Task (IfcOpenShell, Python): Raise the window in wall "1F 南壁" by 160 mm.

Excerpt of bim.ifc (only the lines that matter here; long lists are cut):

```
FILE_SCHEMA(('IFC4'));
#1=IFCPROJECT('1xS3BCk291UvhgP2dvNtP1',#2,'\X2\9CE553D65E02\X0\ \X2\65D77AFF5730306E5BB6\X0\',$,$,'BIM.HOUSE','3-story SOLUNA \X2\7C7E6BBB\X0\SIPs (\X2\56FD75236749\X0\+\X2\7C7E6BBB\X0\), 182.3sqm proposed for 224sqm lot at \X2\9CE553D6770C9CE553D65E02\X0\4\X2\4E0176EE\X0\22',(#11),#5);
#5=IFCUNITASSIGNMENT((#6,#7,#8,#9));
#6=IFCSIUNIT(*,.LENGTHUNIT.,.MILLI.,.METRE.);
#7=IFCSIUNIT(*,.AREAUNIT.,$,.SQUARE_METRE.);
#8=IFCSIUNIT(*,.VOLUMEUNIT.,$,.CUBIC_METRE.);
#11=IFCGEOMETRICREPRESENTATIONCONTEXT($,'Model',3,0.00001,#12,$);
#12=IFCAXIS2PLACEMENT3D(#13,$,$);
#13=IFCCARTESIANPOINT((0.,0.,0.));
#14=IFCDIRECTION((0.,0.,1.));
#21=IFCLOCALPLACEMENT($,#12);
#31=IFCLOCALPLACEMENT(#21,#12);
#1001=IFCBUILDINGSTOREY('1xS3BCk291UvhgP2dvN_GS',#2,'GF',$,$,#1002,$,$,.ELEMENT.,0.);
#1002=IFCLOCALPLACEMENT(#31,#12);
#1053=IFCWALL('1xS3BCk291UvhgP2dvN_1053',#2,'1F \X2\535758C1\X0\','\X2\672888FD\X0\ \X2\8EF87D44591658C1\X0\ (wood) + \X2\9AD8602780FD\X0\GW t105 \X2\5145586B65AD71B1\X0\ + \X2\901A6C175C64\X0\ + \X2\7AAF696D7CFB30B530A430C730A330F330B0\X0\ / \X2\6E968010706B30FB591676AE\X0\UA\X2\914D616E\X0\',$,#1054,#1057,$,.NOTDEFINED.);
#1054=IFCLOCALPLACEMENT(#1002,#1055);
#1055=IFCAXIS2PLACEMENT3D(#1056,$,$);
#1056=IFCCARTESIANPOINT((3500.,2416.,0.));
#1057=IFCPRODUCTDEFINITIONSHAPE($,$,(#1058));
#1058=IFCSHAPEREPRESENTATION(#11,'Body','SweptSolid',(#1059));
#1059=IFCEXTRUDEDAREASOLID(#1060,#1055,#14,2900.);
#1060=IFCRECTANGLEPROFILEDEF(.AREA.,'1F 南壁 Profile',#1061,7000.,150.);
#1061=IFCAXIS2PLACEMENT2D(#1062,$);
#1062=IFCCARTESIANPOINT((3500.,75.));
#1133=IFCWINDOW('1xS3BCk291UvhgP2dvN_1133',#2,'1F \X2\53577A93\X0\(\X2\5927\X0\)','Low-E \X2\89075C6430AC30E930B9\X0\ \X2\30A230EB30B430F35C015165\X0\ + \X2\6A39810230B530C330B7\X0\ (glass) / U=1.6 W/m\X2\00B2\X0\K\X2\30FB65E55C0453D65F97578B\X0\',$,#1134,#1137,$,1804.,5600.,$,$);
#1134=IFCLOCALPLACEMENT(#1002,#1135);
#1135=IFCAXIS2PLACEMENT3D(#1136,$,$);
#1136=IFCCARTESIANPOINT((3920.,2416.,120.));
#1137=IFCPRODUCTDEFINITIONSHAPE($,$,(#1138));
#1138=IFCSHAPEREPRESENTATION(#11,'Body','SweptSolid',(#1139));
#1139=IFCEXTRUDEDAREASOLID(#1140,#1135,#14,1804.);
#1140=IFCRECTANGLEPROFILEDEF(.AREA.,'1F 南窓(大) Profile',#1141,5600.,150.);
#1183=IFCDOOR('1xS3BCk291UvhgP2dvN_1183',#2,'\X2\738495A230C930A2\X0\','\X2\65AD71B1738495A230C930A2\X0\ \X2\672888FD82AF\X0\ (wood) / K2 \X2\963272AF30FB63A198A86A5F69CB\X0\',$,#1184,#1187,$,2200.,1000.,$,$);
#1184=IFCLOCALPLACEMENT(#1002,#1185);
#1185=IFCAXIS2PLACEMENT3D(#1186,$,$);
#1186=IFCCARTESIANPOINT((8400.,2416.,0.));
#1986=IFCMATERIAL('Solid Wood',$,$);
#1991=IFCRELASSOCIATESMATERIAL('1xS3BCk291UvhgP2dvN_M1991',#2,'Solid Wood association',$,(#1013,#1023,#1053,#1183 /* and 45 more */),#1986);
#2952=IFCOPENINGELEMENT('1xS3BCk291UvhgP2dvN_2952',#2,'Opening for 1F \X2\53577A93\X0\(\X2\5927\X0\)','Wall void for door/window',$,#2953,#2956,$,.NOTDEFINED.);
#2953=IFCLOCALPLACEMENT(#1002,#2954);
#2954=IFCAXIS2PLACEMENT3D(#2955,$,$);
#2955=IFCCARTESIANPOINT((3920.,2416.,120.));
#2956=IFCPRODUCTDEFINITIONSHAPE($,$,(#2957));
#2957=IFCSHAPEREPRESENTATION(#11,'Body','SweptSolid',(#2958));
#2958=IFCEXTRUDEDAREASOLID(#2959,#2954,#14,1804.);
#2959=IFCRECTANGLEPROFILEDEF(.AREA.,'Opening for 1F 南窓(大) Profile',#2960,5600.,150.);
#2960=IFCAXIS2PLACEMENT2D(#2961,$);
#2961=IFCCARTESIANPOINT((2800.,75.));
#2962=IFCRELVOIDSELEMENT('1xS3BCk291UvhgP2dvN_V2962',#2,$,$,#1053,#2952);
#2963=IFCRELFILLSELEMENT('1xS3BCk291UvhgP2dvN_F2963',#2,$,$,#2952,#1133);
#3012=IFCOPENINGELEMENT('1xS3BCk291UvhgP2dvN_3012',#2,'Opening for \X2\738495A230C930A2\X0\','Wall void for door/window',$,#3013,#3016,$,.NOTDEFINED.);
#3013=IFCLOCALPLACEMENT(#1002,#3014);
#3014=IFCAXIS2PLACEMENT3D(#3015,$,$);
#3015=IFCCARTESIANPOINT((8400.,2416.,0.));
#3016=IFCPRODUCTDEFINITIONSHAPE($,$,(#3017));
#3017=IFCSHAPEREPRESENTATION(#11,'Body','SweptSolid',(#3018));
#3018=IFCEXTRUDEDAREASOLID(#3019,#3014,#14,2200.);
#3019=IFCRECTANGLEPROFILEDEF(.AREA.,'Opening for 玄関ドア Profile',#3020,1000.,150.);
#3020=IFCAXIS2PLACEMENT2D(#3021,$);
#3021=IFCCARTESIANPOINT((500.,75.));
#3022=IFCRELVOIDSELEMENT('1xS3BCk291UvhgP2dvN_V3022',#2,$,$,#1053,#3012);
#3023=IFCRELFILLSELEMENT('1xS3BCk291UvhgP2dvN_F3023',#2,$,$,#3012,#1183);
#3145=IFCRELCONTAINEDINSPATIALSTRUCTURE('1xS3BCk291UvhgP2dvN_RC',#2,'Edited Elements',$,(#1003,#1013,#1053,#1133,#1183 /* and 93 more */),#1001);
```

```python
import numpy as np
import ifcopenshell
import ifcopenshell.api.geometry
import ifcopenshell.util.placement
import ifcopenshell.util.unit

model = ifcopenshell.open("bim.ifc")
unit_scale = ifcopenshell.util.unit.calculate_unit_scale(model)

window = model.by_id(1133)
opening = window.FillsVoids[0].RelatingOpeningElement
dz = 160.0

shift = np.array([0.0, 0.0, dz])
# The window is not placed relative to its opening, so move both.
for product in (opening, window):
    matrix = ifcopenshell.util.placement.get_local_placement(product.ObjectPlacement)
    matrix[:3, 3] += shift
    ifcopenshell.api.geometry.edit_object_placement(model, product=product, matrix=matrix, is_si=False)

print(f"moved by {dz * unit_scale:+.3f} m")

model.write("bim_v2.ifc")
```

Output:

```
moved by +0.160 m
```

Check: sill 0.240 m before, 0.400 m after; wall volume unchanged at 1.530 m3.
